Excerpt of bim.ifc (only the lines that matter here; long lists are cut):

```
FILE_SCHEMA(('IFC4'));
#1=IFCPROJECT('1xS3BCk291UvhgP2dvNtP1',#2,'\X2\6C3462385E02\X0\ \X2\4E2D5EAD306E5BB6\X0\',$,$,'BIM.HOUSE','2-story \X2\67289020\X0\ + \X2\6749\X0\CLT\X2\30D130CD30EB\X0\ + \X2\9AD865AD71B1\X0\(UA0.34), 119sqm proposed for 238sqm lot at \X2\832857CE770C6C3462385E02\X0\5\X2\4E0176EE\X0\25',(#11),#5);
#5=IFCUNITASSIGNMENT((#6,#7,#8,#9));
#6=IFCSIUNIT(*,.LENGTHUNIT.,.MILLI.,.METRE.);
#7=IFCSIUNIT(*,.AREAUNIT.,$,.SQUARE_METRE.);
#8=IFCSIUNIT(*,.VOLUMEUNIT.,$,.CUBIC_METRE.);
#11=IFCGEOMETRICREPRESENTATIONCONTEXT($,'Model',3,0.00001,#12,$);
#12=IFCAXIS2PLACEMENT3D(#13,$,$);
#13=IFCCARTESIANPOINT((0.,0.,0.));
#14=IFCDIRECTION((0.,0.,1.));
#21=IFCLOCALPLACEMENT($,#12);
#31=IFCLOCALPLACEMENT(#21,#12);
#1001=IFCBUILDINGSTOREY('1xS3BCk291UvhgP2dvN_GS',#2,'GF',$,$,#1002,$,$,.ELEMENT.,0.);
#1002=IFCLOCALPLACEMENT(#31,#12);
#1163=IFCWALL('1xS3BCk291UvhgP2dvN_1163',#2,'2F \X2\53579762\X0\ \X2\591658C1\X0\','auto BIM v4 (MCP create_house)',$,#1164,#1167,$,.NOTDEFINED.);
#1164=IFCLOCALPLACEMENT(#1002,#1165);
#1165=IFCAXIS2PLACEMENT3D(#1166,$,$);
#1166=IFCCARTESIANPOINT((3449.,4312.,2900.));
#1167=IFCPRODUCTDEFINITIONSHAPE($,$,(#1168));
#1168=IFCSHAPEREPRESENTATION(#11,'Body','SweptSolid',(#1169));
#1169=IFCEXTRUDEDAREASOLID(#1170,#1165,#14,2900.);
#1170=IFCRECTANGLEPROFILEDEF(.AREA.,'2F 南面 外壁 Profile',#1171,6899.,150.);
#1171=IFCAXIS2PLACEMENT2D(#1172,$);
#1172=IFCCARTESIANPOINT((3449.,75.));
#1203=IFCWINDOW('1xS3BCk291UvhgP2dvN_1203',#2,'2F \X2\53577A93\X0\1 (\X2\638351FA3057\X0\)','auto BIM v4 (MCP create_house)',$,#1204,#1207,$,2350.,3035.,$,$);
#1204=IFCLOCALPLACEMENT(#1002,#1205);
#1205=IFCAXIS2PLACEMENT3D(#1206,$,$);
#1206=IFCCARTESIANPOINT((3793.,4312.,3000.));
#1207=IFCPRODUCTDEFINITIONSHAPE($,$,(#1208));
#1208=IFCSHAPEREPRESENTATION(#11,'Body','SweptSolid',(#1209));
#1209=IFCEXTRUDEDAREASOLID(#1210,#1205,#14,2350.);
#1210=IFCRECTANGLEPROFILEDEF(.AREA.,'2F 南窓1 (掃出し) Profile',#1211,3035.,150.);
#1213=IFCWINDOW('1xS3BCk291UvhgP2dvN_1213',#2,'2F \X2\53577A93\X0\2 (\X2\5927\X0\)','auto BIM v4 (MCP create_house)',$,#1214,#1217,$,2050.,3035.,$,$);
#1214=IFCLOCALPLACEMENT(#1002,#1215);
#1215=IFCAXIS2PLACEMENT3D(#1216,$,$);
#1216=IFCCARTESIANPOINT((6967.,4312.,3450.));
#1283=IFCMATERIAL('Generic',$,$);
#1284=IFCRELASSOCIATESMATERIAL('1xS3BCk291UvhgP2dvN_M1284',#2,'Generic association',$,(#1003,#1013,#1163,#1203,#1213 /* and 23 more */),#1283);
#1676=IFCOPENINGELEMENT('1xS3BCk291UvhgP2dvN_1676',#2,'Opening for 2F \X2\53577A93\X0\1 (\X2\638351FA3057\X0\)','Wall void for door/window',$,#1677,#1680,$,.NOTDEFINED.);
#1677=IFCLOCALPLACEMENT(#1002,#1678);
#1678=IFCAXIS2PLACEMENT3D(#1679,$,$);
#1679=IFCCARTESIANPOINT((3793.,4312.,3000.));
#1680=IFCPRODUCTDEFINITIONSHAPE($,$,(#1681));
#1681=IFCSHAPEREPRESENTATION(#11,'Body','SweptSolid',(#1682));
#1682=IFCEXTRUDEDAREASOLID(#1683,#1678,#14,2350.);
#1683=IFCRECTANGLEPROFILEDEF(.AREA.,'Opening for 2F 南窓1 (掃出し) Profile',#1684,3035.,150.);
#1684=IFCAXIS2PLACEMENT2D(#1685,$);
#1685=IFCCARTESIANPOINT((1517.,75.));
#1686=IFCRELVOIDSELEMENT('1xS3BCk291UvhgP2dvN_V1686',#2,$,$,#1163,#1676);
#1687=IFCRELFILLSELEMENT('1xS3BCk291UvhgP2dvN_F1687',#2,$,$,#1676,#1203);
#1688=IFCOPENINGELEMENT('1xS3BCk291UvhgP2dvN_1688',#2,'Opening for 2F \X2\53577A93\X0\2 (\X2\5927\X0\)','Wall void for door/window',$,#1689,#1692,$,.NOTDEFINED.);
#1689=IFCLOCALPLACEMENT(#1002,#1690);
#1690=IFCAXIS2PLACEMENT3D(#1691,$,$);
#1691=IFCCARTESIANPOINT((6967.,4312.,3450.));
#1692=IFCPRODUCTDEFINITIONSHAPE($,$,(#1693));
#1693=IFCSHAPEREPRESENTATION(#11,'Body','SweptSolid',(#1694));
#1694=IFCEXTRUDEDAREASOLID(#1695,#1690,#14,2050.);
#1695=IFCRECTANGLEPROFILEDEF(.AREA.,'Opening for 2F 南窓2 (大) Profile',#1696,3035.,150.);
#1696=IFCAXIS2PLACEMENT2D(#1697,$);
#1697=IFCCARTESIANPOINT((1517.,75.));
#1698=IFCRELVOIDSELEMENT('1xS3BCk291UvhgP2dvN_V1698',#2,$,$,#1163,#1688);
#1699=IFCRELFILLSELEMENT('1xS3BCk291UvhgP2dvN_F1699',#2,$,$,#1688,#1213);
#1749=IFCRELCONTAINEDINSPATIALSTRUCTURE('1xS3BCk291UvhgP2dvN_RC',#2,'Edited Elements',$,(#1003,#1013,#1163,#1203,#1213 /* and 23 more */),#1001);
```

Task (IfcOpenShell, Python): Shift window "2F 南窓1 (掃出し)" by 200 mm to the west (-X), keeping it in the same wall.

```python
import ifcopenshell
import ifcopenshell.api.geometry
import ifcopenshell.util.placement

model = ifcopenshell.open("bim.ifc")

window = model.by_guid("1xS3BCk291UvhgP2dvN_1203")
opening = window.FillsVoids[0].RelatingOpeningElement
wall = opening.VoidsElements[0].RelatingBuildingElement

wall_matrix = ifcopenshell.util.placement.get_local_placement(wall.ObjectPlacement)
shift = wall_matrix[:3, 0] * -200.0
before = ifcopenshell.util.placement.get_local_placement(window.ObjectPlacement)[:3, 3].copy()

# The window is not placed relative to its opening, so move both.
for product in (opening, window):
    matrix = ifcopenshell.util.placement.get_local_placement(product.ObjectPlacement)
    matrix[:3, 3] += shift
    ifcopenshell.api.geometry.edit_object_placement(model, product=product, matrix=matrix, is_si=False)

after = ifcopenshell.util.placement.get_local_placement(window.ObjectPlacement)[:3, 3]
print("window moved by", (after - before).round(3) + 0.0)

model.write("bim_edited.ifc")
```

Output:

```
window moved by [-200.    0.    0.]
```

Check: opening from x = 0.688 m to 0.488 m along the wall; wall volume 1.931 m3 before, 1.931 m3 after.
